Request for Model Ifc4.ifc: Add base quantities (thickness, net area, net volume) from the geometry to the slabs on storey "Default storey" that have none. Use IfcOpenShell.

First a look at what the model holds.

```python
import ifcopenshell
import ifcopenshell.util.element
import ifcopenshell.util.unit

model = ifcopenshell.open("Model Ifc4.ifc")
print(model.schema)
for unit_type in ("LENGTHUNIT", "AREAUNIT", "VOLUMEUNIT"):
    print(unit_type, ifcopenshell.util.unit.calculate_unit_scale(model, unit_type))
storey = next(s for s in model.by_type("IfcBuildingStorey") if s.Name == "Default storey")
slabs = [e for e in ifcopenshell.util.element.get_decomposition(storey) if e.is_a("IfcSlab")]
for e in sorted(slabs, key=lambda e: e.id()):
    print(e.id(), e.is_a(), e.Name, list(ifcopenshell.util.element.get_psets(e, qtos_only=True)), sep=" | ")
```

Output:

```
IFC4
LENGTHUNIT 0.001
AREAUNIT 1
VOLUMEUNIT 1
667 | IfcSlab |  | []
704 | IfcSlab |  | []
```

```python
import ifcopenshell
import ifcopenshell.api.pset
import ifcopenshell.geom
import ifcopenshell.util.element
import ifcopenshell.util.shape
import ifcopenshell.util.unit

model = ifcopenshell.open("Model Ifc4.ifc")
unit_scale = ifcopenshell.util.unit.calculate_unit_scale(model)
area_scale = ifcopenshell.util.unit.calculate_unit_scale(model, "AREAUNIT")
volume_scale = ifcopenshell.util.unit.calculate_unit_scale(model, "VOLUMEUNIT")
settings = ifcopenshell.geom.settings()

storey = next(s for s in model.by_type("IfcBuildingStorey") if s.Name == "Default storey")
slabs = [e for e in ifcopenshell.util.element.get_decomposition(storey) if e.is_a("IfcSlab")]

for e in sorted(slabs, key=lambda e: e.id()):
    if ifcopenshell.util.element.get_psets(e, qtos_only=True, should_inherit=False):
        continue
    # Geometry comes back in metres, in the element's own axes.
    shape = ifcopenshell.geom.create_shape(settings, e)
    values = {
        "Width": ifcopenshell.util.shape.get_z(shape.geometry) / unit_scale,
        "NetArea": ifcopenshell.util.shape.get_footprint_area(shape.geometry) / area_scale,
        "NetVolume": ifcopenshell.util.shape.get_volume(shape.geometry) / volume_scale,
    }
    qto = ifcopenshell.api.pset.add_qto(model, product=e, name="Qto_SlabBaseQuantities")
    ifcopenshell.api.pset.edit_qto(model, qto=qto, properties=values)
    print(e.id(), {k: round(v, 3) for k, v in values.items()})

model.write("Model Ifc4_v2.ifc")
```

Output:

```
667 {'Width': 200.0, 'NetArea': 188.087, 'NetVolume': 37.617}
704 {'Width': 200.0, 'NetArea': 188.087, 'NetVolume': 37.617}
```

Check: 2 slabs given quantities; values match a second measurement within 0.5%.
